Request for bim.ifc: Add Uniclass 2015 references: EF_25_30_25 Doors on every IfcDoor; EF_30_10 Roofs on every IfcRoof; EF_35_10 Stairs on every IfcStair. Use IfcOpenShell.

First a look at what the model holds.

```python
import ifcopenshell

model = ifcopenshell.open("bim.ifc")
print(model.schema)
print("classifications:", [c.Name for c in model.by_type("IfcClassification")])
for ifc_class in ("IfcDoor", "IfcRoof", "IfcStair", "IfcWall", "IfcWindow"):
    print(ifc_class, len(model.by_type(ifc_class)))
```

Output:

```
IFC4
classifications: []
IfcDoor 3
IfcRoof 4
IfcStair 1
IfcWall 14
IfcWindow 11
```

```python
import ifcopenshell
import ifcopenshell.api.classification

model = ifcopenshell.open("bim.ifc")

system = ifcopenshell.api.classification.add_classification(model, classification="Uniclass 2015")

codes = {
    "IfcDoor": ("EF_25_30_25", "Doors"),
    "IfcRoof": ("EF_30_10", "Roofs"),
    "IfcStair": ("EF_35_10", "Stairs"),
}
for ifc_class, (code, name) in codes.items():
    products = model.by_type(ifc_class)
    ifcopenshell.api.classification.add_reference(
        model, products=products, classification=system, identification=code, name=name
    )
    print(code, len(products))

model.write("bim_rev.ifc")
```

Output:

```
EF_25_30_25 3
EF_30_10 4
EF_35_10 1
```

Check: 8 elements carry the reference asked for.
